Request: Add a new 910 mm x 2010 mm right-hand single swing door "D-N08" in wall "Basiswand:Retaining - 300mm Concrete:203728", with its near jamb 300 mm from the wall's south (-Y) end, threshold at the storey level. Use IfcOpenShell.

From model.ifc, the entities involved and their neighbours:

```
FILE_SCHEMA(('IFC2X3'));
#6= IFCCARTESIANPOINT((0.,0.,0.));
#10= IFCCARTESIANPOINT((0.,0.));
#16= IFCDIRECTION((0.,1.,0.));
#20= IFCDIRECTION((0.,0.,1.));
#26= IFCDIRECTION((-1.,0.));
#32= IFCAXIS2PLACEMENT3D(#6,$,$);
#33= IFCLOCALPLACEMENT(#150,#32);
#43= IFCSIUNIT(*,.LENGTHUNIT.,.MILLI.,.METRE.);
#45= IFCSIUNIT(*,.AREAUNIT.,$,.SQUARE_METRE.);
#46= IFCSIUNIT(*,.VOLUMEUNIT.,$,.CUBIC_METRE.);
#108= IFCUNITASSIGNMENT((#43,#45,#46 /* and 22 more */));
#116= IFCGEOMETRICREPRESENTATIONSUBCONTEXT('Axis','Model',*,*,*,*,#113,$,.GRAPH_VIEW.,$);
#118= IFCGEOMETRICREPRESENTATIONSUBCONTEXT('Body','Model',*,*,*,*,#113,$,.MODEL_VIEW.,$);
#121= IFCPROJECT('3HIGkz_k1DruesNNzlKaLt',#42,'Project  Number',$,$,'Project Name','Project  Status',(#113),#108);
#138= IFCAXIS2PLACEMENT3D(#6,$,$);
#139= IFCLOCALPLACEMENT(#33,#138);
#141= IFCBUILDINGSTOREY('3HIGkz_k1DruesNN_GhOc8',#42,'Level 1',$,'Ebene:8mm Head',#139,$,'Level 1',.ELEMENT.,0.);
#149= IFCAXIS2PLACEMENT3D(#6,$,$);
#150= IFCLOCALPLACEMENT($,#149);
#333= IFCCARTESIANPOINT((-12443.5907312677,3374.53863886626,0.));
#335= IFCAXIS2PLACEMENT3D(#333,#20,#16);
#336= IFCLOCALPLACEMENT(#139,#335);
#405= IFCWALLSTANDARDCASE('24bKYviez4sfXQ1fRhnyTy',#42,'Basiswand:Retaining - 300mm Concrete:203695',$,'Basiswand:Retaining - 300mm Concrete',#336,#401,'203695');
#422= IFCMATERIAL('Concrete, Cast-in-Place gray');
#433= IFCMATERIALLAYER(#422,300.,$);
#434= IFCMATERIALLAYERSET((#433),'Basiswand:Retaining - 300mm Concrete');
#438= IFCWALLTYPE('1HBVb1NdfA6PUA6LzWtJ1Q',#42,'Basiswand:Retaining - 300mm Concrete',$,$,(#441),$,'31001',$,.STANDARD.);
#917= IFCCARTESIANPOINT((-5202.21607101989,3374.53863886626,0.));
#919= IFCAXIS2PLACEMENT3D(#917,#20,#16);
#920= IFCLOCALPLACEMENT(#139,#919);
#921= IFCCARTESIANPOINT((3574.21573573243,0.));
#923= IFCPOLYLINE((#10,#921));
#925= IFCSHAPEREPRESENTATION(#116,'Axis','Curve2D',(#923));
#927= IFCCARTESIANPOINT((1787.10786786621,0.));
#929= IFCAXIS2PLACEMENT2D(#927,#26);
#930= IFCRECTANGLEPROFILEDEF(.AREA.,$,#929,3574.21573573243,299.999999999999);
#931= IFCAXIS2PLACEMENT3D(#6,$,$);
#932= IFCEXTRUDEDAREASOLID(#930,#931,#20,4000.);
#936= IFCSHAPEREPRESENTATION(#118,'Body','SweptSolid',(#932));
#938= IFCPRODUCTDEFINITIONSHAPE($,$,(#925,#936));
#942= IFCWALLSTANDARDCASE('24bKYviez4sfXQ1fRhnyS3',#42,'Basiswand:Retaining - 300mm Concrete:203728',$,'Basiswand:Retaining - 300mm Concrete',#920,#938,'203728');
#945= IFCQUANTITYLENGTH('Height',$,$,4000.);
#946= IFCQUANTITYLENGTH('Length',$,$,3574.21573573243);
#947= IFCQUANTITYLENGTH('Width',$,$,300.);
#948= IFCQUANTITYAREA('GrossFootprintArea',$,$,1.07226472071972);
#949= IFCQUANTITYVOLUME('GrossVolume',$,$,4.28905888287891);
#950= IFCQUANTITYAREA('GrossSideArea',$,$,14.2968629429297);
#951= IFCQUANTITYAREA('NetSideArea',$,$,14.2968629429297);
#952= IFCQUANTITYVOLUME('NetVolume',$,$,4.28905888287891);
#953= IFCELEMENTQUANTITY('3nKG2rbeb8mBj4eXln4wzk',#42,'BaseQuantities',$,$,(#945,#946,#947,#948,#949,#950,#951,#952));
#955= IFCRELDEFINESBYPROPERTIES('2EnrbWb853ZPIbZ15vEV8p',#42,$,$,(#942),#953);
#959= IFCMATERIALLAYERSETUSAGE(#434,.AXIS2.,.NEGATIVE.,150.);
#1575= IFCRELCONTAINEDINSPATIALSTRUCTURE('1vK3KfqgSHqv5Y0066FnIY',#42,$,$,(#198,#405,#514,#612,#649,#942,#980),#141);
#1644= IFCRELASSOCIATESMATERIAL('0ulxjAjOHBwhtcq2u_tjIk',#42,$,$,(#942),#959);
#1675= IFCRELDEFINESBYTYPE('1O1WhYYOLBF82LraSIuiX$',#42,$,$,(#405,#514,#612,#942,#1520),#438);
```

```python
import numpy as np
import ifcopenshell
import ifcopenshell.api.feature
import ifcopenshell.api.geometry
import ifcopenshell.api.pset
import ifcopenshell.api.root
import ifcopenshell.api.spatial
import ifcopenshell.api.type
import ifcopenshell.geom
import ifcopenshell.util.element
import ifcopenshell.util.placement
import ifcopenshell.util.representation
import ifcopenshell.util.shape
import ifcopenshell.util.unit

model = ifcopenshell.open("model.ifc")
unit_scale = ifcopenshell.util.unit.calculate_unit_scale(model)
area_scale = ifcopenshell.util.unit.calculate_unit_scale(model, "AREAUNIT")
volume_scale = ifcopenshell.util.unit.calculate_unit_scale(model, "VOLUMEUNIT")
settings = ifcopenshell.geom.settings()


def volume(element):
    """Net volume in cubic metres, openings subtracted."""
    shape = ifcopenshell.geom.create_shape(settings, element)
    return ifcopenshell.util.shape.get_volume(shape.geometry)


wall = model.by_guid("24bKYviez4sfXQ1fRhnyS3")
storey = ifcopenshell.util.element.get_container(wall, ifc_class="IfcBuildingStorey")
context = ifcopenshell.util.representation.get_context(model, "Model", "Body", "MODEL_VIEW")
before = volume(wall)

width, height, from_end, sill = 0.91, 2.01, 0.3, 0.0  # metres

# The wall runs along its own X axis, and the end named is its -X end.
wall_shape = ifcopenshell.geom.create_shape(settings, wall)
x, y, z = ifcopenshell.util.shape.get_vertices(wall_shape.geometry).T
start = x.min() + from_end
face, thickness = float(y.min()), float(y.max() - y.min())
wall_matrix = ifcopenshell.util.placement.get_local_placement(wall.ObjectPlacement)
level = ifcopenshell.util.placement.get_local_placement(storey.ObjectPlacement)[2, 3]


def in_wall(x, y):
    """Placement at x, y metres in the wall's axes, at sill height."""
    matrix = wall_matrix.copy()
    matrix[:, 3] = wall_matrix @ np.array([x / unit_scale, y / unit_scale, 0.0, 1.0])
    matrix[2, 3] = level + sill / unit_scale
    return matrix


# Opening: a box that overshoots both wall faces by 50 mm.
opening = ifcopenshell.api.root.create_entity(model, ifc_class="IfcOpeningElement")
box = ifcopenshell.api.geometry.add_wall_representation(
    model, context=context, length=width, height=height, thickness=thickness + 0.1
)
ifcopenshell.api.geometry.assign_representation(model, product=opening, representation=box)
ifcopenshell.api.geometry.edit_object_placement(model, product=opening, matrix=in_wall(start, face - 0.05), is_si=False)
ifcopenshell.api.feature.add_feature(model, feature=opening, element=wall)

door = ifcopenshell.api.root.create_entity(model, ifc_class="IfcDoor", name="D-N08")
door.OverallWidth, door.OverallHeight = width / unit_scale, height / unit_scale
body = ifcopenshell.api.geometry.add_door_representation(
    model,
    context=context,
    overall_width=door.OverallWidth,
    overall_height=door.OverallHeight,
    operation_type="SINGLE_SWING_RIGHT",
    lining_properties={"LiningDepth": thickness / unit_scale, "ThresholdDepth": thickness / unit_scale},
)
ifcopenshell.api.geometry.assign_representation(model, product=door, representation=body)
ifcopenshell.api.spatial.assign_container(model, products=[door], relating_structure=storey)
fills = ifcopenshell.api.feature.add_filling(model, opening=opening, element=door)
fills.OwnerHistory = door.OwnerHistory  # required in IFC2X3

# IFC2X3 keeps the operation on the door style.
style = ifcopenshell.api.root.create_entity(model, ifc_class="IfcDoorStyle", name="D-N08")
style.OperationType, style.ConstructionType = "SINGLE_SWING_RIGHT", "NOTDEFINED"
style.ParameterTakesPrecedence = style.Sizeable = False
ifcopenshell.api.type.assign_type(model, related_objects=[door], relating_type=style)

# The lining spans the wall, so the door starts at the wall face.
ifcopenshell.api.geometry.edit_object_placement(model, product=door, matrix=in_wall(start, face), is_si=False)

after = volume(wall)

# Update the wall's stored quantities.
qto = model.by_id(ifcopenshell.util.element.get_pset(wall, "BaseQuantities", should_inherit=False)["id"])
ifcopenshell.api.pset.edit_qto(model, qto=qto, properties={
    "NetSideArea": after / thickness / area_scale,
    "NetVolume": after / volume_scale,
})

print(f"wall volume {before:.3f} -> {after:.3f} m3")

model.write("model_v2.ifc")
```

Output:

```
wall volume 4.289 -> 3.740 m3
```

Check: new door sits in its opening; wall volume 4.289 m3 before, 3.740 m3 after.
